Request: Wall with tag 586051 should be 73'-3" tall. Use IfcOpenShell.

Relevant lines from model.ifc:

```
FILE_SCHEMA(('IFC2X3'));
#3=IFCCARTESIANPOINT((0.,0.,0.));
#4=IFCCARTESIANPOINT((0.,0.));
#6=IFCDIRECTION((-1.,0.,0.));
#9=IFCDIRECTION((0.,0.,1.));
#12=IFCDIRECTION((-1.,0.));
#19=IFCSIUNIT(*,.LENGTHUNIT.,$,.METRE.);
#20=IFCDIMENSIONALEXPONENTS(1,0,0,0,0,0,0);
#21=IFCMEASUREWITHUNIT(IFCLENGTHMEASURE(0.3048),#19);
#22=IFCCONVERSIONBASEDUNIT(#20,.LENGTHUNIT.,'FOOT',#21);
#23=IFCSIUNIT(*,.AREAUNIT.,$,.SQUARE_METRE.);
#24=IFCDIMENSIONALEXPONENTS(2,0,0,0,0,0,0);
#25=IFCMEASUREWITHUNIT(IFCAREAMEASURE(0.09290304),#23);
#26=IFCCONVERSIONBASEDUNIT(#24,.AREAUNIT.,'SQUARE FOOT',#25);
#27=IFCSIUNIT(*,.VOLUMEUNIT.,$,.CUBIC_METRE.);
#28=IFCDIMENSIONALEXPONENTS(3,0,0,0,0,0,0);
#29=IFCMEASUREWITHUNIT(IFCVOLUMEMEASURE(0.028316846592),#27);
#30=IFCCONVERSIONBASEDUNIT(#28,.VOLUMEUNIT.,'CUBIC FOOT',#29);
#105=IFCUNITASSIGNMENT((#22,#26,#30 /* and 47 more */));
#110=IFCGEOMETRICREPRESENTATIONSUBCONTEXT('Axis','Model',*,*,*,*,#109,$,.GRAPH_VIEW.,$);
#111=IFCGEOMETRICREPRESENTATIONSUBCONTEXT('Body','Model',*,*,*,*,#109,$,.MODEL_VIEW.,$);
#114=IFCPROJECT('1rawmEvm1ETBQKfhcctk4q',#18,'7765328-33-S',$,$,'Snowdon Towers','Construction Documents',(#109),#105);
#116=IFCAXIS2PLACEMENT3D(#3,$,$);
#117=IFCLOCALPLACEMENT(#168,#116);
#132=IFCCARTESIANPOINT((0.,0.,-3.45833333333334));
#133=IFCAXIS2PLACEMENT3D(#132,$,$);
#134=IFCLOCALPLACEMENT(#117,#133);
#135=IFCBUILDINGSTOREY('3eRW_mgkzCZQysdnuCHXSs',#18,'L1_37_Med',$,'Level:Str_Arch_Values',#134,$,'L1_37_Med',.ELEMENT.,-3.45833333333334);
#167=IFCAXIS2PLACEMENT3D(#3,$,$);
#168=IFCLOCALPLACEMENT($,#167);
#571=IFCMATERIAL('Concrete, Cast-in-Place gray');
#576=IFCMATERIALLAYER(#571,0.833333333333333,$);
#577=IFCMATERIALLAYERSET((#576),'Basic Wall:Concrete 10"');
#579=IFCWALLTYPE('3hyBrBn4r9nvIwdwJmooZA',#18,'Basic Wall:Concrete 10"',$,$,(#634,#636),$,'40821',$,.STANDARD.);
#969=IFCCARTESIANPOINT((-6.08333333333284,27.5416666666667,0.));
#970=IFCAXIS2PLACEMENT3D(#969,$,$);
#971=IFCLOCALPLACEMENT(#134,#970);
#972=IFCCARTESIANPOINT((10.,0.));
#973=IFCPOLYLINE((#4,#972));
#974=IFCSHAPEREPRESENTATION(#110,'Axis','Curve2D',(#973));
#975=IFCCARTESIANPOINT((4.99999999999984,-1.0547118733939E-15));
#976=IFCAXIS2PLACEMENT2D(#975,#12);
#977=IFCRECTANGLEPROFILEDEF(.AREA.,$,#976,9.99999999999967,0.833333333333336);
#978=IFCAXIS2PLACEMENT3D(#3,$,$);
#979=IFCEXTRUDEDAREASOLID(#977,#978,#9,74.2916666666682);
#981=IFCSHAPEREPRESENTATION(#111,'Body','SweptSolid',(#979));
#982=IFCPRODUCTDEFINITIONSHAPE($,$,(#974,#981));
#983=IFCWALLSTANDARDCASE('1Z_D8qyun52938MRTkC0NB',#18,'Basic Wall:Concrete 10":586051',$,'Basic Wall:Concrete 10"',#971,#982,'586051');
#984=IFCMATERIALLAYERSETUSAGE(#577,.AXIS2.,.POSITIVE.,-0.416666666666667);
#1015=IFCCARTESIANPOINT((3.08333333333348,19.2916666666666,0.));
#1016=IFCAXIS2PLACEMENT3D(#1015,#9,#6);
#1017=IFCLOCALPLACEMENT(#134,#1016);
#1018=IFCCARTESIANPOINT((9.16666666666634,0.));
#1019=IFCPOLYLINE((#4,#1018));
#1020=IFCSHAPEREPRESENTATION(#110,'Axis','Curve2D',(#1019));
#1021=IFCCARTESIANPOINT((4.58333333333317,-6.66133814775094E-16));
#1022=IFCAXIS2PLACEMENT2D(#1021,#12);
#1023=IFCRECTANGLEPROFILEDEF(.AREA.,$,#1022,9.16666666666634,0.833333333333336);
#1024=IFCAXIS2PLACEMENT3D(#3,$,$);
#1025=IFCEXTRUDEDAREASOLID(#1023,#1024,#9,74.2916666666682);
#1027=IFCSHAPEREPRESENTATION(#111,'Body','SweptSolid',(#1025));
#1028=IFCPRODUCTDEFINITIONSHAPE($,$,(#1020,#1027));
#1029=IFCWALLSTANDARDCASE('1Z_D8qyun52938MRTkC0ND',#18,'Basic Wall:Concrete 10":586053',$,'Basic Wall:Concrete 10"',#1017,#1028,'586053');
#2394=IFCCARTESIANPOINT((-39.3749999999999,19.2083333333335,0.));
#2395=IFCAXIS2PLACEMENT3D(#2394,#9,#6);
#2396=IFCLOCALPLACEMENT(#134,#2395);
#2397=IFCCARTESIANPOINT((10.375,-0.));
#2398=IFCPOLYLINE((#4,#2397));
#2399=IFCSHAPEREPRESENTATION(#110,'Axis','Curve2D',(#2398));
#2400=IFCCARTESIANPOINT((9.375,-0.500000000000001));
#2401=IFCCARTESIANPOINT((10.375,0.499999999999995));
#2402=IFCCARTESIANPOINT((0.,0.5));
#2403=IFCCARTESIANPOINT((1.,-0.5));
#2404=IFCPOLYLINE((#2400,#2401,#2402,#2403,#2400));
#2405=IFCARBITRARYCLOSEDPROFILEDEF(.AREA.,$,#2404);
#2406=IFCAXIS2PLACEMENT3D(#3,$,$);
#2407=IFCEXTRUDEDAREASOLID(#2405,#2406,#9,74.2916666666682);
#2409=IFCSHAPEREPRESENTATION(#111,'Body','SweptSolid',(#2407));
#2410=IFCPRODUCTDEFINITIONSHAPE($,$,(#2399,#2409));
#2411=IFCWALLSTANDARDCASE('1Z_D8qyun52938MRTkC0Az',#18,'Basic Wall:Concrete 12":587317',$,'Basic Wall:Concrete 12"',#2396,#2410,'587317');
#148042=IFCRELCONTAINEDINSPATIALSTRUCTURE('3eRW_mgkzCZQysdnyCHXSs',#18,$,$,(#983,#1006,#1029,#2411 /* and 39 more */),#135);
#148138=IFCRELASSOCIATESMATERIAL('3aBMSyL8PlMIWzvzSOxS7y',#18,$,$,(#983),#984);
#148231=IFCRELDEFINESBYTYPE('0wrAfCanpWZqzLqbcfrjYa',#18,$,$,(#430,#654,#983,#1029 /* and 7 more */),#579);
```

```python
import ifcopenshell
import ifcopenshell.geom
import ifcopenshell.util.representation
import ifcopenshell.util.shape
import ifcopenshell.util.unit

model = ifcopenshell.open("model.ifc")
unit_scale = ifcopenshell.util.unit.calculate_unit_scale(model)
settings = ifcopenshell.geom.settings()


def volume(element):
    """Net volume in cubic metres, openings subtracted."""
    shape = ifcopenshell.geom.create_shape(settings, element)
    return ifcopenshell.util.shape.get_volume(shape.geometry)


wall = model.by_guid("1Z_D8qyun52938MRTkC0NB")
before = volume(wall)

body = ifcopenshell.util.representation.get_representation(wall, "Model", "Body")
solid = body.Items[0]
old_height = solid.Depth
solid.Depth = 879 * 0.0254 / unit_scale
after = volume(wall)

print(f"height {old_height:g} -> {solid.Depth:g}, volume {before:.3f} -> {after:.3f} m3")

model.write("model_rev.ifc")
```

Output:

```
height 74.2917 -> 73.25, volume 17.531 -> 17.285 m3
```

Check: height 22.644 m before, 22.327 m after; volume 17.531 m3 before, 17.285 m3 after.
